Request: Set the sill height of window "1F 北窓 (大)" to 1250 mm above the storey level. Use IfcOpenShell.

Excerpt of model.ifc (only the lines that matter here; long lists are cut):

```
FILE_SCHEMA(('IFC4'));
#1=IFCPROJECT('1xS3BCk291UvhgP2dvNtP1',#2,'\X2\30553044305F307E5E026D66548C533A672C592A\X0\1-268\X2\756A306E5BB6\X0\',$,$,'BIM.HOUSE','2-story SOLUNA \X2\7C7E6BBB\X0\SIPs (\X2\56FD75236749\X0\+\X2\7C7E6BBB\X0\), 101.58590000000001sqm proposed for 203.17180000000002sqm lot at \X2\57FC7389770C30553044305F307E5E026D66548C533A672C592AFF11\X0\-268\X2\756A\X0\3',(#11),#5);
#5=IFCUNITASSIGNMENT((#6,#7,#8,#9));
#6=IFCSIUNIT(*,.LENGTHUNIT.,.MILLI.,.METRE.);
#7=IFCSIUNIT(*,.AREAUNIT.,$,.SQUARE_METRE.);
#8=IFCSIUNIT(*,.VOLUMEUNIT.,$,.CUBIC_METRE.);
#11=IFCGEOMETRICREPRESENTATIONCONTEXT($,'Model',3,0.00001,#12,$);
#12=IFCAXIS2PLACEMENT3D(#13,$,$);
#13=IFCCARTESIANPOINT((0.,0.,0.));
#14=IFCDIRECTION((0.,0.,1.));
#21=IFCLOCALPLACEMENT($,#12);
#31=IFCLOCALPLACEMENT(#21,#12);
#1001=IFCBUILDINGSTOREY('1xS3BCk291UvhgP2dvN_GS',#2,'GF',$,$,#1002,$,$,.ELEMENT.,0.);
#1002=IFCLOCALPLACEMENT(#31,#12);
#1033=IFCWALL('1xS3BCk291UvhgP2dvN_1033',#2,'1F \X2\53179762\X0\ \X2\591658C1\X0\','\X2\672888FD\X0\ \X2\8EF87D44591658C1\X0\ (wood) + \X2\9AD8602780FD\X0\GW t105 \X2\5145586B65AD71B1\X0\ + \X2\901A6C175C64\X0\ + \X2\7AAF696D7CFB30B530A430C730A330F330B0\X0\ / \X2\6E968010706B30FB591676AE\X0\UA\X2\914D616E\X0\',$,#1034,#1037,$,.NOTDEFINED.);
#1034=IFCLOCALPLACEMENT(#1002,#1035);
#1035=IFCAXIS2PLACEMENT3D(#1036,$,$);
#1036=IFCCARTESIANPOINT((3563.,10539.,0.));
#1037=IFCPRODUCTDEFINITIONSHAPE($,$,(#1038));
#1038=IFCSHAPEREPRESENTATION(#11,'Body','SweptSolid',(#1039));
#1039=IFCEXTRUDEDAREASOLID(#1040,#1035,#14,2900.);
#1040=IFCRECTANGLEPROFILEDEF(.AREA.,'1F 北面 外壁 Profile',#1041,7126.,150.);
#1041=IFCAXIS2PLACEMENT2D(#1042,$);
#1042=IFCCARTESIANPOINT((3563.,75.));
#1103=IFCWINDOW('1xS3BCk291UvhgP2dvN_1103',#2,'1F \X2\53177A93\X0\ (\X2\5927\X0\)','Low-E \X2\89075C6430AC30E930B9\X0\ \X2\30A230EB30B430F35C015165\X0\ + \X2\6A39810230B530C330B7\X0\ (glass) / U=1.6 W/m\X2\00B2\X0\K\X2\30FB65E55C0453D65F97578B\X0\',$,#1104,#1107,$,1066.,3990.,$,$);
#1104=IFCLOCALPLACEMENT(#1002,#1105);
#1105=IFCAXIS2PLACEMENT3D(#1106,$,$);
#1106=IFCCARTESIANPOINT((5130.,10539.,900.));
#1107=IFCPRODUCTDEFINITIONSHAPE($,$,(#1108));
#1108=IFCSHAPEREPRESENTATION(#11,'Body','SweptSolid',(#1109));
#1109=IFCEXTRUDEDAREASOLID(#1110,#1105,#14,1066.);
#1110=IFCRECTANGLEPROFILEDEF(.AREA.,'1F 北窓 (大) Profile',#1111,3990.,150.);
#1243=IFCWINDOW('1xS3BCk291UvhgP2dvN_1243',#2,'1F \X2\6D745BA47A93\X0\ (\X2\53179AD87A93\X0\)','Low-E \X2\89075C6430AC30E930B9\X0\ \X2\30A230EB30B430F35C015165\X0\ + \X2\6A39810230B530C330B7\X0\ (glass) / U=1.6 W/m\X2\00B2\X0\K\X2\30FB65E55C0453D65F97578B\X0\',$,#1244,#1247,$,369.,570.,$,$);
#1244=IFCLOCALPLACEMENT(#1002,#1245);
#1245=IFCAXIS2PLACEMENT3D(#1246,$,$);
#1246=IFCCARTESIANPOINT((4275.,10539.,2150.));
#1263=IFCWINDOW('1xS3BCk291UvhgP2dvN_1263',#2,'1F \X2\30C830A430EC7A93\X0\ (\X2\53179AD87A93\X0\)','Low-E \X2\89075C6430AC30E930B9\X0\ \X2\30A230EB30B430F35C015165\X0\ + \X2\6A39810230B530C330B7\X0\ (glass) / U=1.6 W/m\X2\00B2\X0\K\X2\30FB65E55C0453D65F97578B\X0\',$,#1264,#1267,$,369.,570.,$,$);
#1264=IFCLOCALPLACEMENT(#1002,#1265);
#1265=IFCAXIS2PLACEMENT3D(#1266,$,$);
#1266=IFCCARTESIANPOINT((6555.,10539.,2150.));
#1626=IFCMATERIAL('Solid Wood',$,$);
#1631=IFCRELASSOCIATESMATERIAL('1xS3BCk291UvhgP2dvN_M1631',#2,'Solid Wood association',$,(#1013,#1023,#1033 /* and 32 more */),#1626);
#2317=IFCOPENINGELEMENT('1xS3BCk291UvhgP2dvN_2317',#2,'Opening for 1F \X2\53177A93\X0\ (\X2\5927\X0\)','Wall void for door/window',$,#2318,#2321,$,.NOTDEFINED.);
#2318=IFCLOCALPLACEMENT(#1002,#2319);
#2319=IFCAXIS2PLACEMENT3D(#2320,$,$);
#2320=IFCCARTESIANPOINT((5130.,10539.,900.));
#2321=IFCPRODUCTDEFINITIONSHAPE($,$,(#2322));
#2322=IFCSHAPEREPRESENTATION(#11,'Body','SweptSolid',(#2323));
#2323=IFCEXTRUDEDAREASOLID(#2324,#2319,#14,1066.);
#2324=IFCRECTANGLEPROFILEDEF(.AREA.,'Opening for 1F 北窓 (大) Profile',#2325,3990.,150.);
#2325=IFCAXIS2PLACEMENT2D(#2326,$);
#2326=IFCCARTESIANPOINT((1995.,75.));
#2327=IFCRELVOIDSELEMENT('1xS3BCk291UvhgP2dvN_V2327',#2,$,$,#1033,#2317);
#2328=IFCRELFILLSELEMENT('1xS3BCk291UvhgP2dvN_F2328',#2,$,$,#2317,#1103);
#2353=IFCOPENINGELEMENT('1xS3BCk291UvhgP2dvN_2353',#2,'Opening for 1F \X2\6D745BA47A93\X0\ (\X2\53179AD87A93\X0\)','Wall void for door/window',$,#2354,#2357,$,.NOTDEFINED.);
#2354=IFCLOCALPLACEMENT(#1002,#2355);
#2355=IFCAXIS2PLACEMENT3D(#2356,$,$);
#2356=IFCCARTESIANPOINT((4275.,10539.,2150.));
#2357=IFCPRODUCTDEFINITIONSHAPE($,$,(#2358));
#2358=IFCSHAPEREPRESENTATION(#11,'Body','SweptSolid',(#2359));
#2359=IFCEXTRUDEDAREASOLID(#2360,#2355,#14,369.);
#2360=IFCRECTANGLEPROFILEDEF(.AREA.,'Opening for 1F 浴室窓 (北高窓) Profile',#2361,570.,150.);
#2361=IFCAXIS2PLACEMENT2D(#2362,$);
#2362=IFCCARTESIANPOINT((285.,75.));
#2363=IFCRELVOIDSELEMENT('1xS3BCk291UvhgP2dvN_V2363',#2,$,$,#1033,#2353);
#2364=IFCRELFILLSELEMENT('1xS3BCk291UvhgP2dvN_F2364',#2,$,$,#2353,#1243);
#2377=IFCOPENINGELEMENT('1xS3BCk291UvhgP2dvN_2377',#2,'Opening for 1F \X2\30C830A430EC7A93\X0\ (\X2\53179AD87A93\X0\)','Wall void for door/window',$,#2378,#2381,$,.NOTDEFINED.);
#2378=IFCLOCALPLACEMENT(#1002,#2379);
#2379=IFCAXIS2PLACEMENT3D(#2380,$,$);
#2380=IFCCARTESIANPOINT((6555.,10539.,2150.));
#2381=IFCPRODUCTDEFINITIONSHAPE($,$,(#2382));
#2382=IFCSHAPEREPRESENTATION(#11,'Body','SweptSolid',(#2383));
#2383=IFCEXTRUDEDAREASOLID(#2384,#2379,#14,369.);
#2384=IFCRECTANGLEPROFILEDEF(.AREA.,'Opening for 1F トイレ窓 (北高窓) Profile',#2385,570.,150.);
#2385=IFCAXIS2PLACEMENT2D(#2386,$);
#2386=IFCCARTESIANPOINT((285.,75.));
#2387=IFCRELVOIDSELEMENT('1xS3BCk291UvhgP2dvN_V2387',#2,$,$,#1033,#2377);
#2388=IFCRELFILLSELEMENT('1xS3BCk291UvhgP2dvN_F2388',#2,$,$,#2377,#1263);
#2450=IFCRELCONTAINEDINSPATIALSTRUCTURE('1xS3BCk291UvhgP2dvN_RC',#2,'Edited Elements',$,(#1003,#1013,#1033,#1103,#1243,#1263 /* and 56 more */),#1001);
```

```python
import numpy as np
import ifcopenshell
import ifcopenshell.api.geometry
import ifcopenshell.geom
import ifcopenshell.util.element
import ifcopenshell.util.placement
import ifcopenshell.util.shape
import ifcopenshell.util.unit

model = ifcopenshell.open("model.ifc")
unit_scale = ifcopenshell.util.unit.calculate_unit_scale(model)

window = model.by_id(1103)
opening = window.FillsVoids[0].RelatingOpeningElement
storey = ifcopenshell.util.element.get_container(window, ifc_class="IfcBuildingStorey")
level = ifcopenshell.util.placement.get_local_placement(storey.ObjectPlacement)[2, 3]

# The opening's origin need not be at the sill, so measure its lowest point.
shape = ifcopenshell.geom.create_shape(ifcopenshell.geom.settings(), opening)
bottom = ifcopenshell.util.shape.get_shape_bottom_elevation(shape, shape.geometry) / unit_scale
dz = level + 1250.0 - bottom

shift = np.array([0.0, 0.0, dz])
# The window is not placed relative to its opening, so move both.
for product in (opening, window):
    matrix = ifcopenshell.util.placement.get_local_placement(product.ObjectPlacement)
    matrix[:3, 3] += shift
    ifcopenshell.api.geometry.edit_object_placement(model, product=product, matrix=matrix, is_si=False)

print(f"moved by {dz * unit_scale:+.3f} m")

model.write("model_v2.ifc")
```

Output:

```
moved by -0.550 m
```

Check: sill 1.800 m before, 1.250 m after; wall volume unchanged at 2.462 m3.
